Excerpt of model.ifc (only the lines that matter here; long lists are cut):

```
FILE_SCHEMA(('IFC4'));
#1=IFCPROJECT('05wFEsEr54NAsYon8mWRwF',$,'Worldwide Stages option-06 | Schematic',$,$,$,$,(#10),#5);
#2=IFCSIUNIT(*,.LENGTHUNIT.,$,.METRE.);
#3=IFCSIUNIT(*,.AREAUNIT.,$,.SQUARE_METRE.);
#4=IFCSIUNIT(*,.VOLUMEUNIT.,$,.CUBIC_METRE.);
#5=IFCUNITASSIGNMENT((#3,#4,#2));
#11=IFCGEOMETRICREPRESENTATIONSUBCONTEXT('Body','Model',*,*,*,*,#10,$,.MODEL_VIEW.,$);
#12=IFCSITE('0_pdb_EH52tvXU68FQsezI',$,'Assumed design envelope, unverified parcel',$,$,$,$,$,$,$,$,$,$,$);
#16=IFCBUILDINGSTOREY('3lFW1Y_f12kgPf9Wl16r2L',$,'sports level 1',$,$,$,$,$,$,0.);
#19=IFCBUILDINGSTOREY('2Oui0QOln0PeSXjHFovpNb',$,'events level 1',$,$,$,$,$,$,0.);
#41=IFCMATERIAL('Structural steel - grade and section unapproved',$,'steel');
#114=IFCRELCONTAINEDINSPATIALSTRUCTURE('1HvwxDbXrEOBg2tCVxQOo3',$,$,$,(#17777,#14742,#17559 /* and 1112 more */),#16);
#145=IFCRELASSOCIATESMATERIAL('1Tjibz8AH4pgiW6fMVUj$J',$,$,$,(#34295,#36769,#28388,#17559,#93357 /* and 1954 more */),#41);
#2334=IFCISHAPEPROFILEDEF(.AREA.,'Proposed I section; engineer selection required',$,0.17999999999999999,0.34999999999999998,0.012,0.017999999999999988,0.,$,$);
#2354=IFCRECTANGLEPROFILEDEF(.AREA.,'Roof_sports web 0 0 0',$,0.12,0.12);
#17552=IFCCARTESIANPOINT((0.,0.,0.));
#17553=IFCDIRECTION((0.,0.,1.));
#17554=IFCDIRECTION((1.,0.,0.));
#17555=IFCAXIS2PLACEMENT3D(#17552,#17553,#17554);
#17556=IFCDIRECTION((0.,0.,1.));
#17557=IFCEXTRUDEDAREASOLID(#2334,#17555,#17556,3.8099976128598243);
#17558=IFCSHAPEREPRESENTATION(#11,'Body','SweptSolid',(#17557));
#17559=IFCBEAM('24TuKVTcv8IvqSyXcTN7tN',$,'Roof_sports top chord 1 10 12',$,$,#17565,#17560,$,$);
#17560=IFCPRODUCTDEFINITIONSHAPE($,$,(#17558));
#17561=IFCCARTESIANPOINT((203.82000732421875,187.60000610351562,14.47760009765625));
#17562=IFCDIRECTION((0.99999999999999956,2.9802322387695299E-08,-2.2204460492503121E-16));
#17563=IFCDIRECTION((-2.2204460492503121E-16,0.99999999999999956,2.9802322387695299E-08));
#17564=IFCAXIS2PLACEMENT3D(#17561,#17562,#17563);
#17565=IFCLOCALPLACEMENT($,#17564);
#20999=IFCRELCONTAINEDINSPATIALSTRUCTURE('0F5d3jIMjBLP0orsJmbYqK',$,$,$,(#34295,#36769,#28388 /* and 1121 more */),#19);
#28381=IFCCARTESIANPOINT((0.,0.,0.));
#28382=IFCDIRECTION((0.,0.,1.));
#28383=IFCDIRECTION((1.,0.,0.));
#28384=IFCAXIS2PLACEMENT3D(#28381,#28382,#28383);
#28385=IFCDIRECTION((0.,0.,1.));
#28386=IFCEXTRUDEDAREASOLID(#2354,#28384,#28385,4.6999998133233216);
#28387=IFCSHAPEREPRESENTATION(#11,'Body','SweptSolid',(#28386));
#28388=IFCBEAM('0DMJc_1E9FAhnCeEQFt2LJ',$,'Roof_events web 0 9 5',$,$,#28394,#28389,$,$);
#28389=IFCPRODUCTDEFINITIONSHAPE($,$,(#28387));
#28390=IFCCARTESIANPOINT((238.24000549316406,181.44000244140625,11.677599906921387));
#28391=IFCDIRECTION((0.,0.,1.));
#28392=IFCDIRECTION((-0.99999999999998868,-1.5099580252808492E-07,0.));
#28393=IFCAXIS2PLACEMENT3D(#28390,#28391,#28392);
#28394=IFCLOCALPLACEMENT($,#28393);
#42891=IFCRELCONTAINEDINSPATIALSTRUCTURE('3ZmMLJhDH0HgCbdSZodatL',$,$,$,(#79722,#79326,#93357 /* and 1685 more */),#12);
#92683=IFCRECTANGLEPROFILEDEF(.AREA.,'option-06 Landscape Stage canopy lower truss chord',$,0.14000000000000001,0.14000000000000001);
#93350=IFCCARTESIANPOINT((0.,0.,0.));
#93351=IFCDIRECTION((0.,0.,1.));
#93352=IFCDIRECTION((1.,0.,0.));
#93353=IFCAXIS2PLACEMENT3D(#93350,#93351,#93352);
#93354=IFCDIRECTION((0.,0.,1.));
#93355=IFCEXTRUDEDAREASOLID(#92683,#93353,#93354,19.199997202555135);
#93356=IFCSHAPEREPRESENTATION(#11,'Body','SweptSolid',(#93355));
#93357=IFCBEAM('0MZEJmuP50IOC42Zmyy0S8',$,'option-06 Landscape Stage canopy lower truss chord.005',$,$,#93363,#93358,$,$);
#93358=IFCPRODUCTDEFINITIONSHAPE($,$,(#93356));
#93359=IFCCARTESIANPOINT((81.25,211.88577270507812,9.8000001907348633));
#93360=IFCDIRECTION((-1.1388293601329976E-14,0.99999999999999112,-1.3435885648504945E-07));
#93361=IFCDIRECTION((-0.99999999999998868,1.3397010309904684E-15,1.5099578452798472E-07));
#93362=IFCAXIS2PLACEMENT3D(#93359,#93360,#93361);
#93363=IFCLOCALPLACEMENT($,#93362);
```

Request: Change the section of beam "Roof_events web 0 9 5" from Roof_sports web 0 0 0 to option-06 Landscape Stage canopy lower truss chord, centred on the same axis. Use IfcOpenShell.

```python
import ifcopenshell
import ifcopenshell.util.element
import ifcopenshell.util.representation

model = ifcopenshell.open("model.ifc")

member = model.by_guid("0DMJc_1E9FAhnCeEQFt2LJ")
source = next(p for p in model.by_type("IfcRectangleProfileDef") if p.ProfileName == "option-06 Landscape Stage canopy lower truss chord")

body = ifcopenshell.util.representation.get_representation(member, "Model", "Body")
solid = body.Items[0]
old_profile = solid.SweptArea

# Copy the section's sizes but keep this member's own profile position.
profile = ifcopenshell.util.element.copy(model, source)
profile.Position = old_profile.Position
solid.SweptArea = profile
if not model.get_total_inverses(old_profile):
    ifcopenshell.util.element.remove_deep2(model, old_profile)

print(solid.SweptArea)

model.write("model_updated.ifc")
```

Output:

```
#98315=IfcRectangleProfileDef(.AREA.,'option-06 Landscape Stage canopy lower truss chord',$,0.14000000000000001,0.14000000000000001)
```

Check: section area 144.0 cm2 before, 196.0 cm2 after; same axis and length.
